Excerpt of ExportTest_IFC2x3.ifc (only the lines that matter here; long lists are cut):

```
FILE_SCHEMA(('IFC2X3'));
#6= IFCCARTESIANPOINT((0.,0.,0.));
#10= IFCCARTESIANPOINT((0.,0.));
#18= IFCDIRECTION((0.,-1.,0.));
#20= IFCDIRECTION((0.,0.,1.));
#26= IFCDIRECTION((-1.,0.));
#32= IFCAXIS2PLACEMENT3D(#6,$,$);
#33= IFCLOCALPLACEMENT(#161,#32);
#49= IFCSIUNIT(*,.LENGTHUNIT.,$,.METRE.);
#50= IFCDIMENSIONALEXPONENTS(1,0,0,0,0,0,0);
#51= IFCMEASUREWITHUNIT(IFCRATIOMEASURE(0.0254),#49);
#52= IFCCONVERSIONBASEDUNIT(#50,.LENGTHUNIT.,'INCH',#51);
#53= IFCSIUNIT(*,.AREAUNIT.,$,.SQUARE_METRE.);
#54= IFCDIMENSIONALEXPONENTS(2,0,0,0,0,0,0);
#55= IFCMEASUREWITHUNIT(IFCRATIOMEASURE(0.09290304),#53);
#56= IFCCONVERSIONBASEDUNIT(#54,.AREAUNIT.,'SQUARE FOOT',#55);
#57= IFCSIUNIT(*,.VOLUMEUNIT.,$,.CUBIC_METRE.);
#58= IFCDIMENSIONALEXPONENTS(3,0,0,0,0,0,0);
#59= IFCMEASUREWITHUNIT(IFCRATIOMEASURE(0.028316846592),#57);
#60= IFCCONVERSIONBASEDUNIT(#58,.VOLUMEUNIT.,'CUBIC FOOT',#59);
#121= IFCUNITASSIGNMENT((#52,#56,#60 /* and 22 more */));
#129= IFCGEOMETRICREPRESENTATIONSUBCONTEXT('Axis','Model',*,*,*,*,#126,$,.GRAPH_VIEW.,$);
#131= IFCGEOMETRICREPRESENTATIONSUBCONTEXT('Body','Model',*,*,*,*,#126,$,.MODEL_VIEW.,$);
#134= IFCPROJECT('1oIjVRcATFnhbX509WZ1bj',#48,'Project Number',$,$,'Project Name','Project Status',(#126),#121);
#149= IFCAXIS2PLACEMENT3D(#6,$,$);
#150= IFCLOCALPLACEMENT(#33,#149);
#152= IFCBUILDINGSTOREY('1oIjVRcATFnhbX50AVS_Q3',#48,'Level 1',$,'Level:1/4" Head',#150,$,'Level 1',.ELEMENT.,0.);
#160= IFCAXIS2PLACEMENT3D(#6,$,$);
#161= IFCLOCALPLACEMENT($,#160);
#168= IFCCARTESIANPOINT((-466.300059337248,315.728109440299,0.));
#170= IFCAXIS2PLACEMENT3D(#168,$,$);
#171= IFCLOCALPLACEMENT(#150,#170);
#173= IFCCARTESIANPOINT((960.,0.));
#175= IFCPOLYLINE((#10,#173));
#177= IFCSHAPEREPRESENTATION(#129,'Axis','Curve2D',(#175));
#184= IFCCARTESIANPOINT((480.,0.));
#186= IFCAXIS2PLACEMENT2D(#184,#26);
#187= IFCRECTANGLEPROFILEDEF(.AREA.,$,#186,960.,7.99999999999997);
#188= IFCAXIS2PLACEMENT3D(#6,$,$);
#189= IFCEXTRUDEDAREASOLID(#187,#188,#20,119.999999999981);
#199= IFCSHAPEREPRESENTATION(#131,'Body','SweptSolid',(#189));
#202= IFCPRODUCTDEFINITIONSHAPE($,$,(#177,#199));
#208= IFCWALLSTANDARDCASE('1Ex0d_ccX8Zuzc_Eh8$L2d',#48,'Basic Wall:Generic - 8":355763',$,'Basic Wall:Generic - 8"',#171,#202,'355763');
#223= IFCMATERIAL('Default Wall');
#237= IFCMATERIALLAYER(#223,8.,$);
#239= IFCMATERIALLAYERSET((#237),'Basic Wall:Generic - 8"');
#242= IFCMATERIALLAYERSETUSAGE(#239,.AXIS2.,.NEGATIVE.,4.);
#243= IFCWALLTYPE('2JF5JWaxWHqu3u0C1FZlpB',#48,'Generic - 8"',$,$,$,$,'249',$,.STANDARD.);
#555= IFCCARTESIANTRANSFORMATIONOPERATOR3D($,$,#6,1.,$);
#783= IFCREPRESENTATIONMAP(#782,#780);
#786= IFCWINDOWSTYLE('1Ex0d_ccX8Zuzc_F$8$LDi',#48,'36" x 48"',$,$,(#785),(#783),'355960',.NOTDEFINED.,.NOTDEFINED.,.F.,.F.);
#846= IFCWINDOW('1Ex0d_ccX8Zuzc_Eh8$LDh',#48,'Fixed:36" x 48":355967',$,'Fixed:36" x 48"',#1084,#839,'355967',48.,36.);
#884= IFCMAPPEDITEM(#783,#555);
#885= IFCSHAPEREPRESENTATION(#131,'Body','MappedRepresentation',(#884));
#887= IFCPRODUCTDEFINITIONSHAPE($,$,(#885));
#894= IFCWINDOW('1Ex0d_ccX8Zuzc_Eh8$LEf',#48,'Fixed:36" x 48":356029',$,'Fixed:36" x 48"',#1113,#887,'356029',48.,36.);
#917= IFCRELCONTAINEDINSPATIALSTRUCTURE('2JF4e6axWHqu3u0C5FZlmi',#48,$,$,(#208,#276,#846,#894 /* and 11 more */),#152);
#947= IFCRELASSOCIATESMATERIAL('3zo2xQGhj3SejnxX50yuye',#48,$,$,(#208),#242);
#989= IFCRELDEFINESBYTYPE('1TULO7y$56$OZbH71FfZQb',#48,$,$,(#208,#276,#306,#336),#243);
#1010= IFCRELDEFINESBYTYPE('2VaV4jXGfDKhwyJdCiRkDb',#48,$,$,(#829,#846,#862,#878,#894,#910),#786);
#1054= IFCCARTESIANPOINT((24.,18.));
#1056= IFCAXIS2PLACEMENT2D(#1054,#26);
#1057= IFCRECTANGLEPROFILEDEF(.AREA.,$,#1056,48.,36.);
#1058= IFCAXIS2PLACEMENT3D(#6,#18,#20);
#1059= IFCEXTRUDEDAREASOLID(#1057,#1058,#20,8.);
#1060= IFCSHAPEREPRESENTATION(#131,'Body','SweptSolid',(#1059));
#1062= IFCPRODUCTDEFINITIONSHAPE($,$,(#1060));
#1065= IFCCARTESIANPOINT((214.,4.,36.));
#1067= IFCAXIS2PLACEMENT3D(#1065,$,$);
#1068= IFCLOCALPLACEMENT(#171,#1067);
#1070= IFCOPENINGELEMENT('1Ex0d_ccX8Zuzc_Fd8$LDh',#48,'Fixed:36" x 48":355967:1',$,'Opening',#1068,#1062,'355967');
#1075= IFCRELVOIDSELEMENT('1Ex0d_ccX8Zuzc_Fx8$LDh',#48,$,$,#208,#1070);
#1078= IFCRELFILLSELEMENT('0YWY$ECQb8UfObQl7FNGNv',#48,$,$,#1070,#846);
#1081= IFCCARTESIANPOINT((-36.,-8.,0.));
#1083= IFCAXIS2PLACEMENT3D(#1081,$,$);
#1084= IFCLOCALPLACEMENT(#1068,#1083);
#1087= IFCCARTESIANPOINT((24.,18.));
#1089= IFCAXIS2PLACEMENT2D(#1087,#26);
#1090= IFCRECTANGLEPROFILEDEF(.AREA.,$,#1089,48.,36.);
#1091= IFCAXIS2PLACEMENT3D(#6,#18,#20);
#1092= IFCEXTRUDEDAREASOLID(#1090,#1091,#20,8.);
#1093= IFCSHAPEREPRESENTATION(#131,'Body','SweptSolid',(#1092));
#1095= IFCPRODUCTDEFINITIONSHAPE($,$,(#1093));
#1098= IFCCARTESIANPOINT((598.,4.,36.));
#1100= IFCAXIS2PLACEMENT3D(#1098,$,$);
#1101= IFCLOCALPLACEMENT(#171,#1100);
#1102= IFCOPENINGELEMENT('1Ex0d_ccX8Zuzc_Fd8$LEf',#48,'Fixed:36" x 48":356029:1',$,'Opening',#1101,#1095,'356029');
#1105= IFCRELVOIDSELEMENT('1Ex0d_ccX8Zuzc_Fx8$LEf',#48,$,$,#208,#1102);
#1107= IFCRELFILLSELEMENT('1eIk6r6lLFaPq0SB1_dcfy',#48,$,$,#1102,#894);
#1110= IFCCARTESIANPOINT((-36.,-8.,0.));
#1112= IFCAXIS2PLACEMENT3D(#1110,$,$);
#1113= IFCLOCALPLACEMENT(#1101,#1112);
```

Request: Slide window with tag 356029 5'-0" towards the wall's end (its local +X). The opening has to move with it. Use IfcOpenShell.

```python
import ifcopenshell
import ifcopenshell.api.geometry
import ifcopenshell.util.placement
import ifcopenshell.util.unit

model = ifcopenshell.open("ExportTest_IFC2x3.ifc")
unit_scale = ifcopenshell.util.unit.calculate_unit_scale(model)

window = model.by_guid("1Ex0d_ccX8Zuzc_Eh8$LEf")
opening = window.FillsVoids[0].RelatingOpeningElement
wall = opening.VoidsElements[0].RelatingBuildingElement

wall_matrix = ifcopenshell.util.placement.get_local_placement(wall.ObjectPlacement)
shift = wall_matrix[:3, 0] * 60 * 0.0254 / unit_scale
before = ifcopenshell.util.placement.get_local_placement(window.ObjectPlacement)[:3, 3].copy()

# The window is placed relative to its opening, so it follows when the opening moves.
matrix = ifcopenshell.util.placement.get_local_placement(opening.ObjectPlacement)
matrix[:3, 3] += shift
ifcopenshell.api.geometry.edit_object_placement(
    model, product=opening, matrix=matrix, is_si=False, should_transform_children=True
)

after = ifcopenshell.util.placement.get_local_placement(window.ObjectPlacement)[:3, 3]
print("window moved by", (after - before).round(3) + 0.0)

model.write("ExportTest_IFC2x3_updated.ifc")
```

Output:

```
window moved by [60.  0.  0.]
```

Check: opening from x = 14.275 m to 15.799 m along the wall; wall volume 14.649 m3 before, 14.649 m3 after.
